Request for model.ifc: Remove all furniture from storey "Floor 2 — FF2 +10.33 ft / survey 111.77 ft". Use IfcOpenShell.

First a look at what the model holds.

```python
import ifcopenshell
import ifcopenshell.util.element

model = ifcopenshell.open("model.ifc")
print(model.schema)
storey = next(s for s in model.by_type("IfcBuildingStorey") if s.Name == "Floor 2 — FF2 +10.33 ft / survey 111.77 ft")
furniture = [e for e in ifcopenshell.util.element.get_decomposition(storey) if e.is_a("IfcFurnishingElement")]
seen = {}
for e in furniture:
    element_type = ifcopenshell.util.element.get_type(e)
    name = element_type.Name if element_type not in (None, e) else None
    seen[name] = seen.get(name, 0) + 1
for name, count in sorted(seen.items(), key=str):
    print(count, "x", name)
```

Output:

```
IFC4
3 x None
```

```python
import ifcopenshell
import ifcopenshell.api.root
import ifcopenshell.util.element

model = ifcopenshell.open("model.ifc")

storey = next(s for s in model.by_type("IfcBuildingStorey") if s.Name == "Floor 2 — FF2 +10.33 ft / survey 111.77 ft")
furniture = [e for e in ifcopenshell.util.element.get_decomposition(storey) if e.is_a("IfcFurnishingElement")]

for e in furniture:
    ifcopenshell.api.root.remove_product(model, product=e)
print(len(furniture), "removed")

model.write("model_v2.ifc")
```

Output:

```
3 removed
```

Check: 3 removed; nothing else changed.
